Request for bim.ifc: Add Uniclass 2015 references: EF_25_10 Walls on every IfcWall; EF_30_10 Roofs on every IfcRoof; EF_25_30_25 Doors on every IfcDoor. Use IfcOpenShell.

First a look at what the model holds.

```python
import ifcopenshell

model = ifcopenshell.open("bim.ifc")
print(model.schema)
print("classifications:", [c.Name for c in model.by_type("IfcClassification")])
for ifc_class in ("IfcDoor", "IfcRoof", "IfcStair", "IfcWall", "IfcWindow"):
    print(ifc_class, len(model.by_type(ifc_class)))
```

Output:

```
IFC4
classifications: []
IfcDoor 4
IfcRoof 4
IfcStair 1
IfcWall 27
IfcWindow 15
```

```python
import ifcopenshell
import ifcopenshell.api.classification

model = ifcopenshell.open("bim.ifc")

system = ifcopenshell.api.classification.add_classification(model, classification="Uniclass 2015")

codes = {
    "IfcWall": ("EF_25_10", "Walls"),
    "IfcRoof": ("EF_30_10", "Roofs"),
    "IfcDoor": ("EF_25_30_25", "Doors"),
}
for ifc_class, (code, name) in codes.items():
    products = model.by_type(ifc_class)
    ifcopenshell.api.classification.add_reference(
        model, products=products, classification=system, identification=code, name=name
    )
    print(code, len(products))

model.write("bim_edited.ifc")
```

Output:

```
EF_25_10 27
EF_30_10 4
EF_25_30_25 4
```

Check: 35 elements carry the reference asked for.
